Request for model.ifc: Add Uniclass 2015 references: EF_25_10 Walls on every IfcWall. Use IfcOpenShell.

First a look at what the model holds.

```python
import ifcopenshell

model = ifcopenshell.open("model.ifc")
print(model.schema)
print("classifications:", [c.Name for c in model.by_type("IfcClassification")])
for ifc_class in ("IfcDoor", "IfcRoof", "IfcStair", "IfcWall", "IfcWindow"):
    print(ifc_class, len(model.by_type(ifc_class)))
```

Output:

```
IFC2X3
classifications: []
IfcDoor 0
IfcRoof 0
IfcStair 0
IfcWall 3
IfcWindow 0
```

```python
import ifcopenshell
import ifcopenshell.api.classification

model = ifcopenshell.open("model.ifc")

# IFC2X3 requires Source and Edition and has no link from the project to the system.
system = model.create_entity("IfcClassification", Source="NBS", Edition="2015", Name="Uniclass 2015")

codes = {
    "IfcWall": ("EF_25_10", "Walls"),
}
for ifc_class, (code, name) in codes.items():
    products = model.by_type(ifc_class)
    ifcopenshell.api.classification.add_reference(
        model, products=products, classification=system, identification=code, name=name
    )
    print(code, len(products))

model.write("model_v2.ifc")
```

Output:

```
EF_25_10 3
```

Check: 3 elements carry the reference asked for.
